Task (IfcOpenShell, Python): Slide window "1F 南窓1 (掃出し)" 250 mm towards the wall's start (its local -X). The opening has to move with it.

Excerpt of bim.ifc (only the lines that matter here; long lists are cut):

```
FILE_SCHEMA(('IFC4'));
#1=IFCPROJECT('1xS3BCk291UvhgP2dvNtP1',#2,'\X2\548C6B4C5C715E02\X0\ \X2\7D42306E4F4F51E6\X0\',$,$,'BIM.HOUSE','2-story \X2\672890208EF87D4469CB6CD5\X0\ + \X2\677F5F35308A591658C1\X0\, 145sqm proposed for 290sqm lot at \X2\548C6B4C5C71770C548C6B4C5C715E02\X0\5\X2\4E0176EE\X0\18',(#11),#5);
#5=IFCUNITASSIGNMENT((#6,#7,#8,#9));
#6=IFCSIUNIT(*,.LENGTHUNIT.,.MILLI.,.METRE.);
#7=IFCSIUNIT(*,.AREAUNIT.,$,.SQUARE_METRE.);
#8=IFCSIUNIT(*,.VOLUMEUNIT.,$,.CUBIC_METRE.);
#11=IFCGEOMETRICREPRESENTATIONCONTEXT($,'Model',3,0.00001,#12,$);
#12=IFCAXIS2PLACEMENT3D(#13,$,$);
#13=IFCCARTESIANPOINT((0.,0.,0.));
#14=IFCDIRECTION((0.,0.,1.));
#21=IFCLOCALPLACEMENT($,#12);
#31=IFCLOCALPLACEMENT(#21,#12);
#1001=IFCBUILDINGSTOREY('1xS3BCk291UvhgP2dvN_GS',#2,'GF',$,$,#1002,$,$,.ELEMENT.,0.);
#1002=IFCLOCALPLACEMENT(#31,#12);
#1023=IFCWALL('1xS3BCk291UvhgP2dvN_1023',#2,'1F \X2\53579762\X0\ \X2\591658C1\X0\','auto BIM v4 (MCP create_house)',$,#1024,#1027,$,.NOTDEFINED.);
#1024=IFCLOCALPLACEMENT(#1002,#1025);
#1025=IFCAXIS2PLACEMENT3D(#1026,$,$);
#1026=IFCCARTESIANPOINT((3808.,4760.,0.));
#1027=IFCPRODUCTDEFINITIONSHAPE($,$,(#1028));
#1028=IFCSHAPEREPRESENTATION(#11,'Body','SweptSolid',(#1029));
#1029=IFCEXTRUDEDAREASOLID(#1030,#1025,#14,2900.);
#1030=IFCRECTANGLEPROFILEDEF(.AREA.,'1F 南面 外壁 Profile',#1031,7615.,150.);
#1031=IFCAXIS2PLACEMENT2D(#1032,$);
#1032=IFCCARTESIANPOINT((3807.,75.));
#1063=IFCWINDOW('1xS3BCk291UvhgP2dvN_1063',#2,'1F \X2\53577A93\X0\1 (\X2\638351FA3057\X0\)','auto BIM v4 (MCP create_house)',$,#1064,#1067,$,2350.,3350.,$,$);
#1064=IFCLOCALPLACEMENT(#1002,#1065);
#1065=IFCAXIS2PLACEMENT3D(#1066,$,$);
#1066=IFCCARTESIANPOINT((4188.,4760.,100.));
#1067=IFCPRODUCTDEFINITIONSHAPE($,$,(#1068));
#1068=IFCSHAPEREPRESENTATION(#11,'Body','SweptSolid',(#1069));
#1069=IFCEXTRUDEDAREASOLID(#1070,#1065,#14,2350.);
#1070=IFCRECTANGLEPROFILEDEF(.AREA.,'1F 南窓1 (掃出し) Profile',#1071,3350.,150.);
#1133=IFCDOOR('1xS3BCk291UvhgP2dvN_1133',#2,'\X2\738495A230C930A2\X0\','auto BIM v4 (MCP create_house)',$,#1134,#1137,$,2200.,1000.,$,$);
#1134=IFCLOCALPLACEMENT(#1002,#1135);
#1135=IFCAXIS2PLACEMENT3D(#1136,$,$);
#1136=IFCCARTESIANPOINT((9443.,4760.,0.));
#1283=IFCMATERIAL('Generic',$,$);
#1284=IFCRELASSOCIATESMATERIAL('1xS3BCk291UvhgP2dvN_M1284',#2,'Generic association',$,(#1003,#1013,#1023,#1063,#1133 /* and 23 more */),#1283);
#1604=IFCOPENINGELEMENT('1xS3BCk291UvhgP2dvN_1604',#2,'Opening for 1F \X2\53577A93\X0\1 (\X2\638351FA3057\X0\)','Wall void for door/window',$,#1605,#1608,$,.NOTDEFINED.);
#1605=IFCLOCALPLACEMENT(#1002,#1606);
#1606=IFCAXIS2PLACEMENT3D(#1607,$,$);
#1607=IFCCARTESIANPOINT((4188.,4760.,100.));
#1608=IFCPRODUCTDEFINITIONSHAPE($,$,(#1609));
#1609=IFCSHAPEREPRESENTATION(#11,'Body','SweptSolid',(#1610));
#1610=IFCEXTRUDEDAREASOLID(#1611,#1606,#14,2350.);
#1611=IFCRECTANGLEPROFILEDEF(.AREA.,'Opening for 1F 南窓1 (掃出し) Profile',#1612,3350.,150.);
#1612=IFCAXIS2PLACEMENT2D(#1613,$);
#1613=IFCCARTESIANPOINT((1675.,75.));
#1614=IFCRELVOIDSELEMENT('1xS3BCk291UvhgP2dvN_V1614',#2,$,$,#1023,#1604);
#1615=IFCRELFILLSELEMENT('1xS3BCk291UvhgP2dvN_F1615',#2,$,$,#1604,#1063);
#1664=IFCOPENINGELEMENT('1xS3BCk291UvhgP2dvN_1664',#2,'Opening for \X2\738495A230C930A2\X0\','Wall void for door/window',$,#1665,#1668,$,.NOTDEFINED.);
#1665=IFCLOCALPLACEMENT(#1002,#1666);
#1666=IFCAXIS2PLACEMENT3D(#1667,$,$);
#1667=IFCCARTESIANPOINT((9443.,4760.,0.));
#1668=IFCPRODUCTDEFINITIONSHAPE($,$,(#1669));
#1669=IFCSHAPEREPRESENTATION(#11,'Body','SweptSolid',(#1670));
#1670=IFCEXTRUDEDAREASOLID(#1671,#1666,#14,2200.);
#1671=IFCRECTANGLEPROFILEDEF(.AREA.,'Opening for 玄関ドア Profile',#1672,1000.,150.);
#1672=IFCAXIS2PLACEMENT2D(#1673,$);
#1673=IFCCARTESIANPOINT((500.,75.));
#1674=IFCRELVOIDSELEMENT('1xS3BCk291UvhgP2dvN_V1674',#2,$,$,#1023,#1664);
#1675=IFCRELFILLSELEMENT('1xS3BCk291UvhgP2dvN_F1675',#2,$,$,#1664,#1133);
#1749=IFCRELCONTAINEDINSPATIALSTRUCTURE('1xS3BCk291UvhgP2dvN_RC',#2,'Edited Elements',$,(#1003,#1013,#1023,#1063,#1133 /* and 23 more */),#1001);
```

```python
import ifcopenshell
import ifcopenshell.api.geometry
import ifcopenshell.util.placement
import ifcopenshell.util.unit

model = ifcopenshell.open("bim.ifc")
unit_scale = ifcopenshell.util.unit.calculate_unit_scale(model)

window = model.by_guid("1xS3BCk291UvhgP2dvN_1063")
opening = window.FillsVoids[0].RelatingOpeningElement
wall = opening.VoidsElements[0].RelatingBuildingElement

wall_matrix = ifcopenshell.util.placement.get_local_placement(wall.ObjectPlacement)
shift = wall_matrix[:3, 0] * -0.25 / unit_scale
before = ifcopenshell.util.placement.get_local_placement(window.ObjectPlacement)[:3, 3].copy()

# The window is not placed relative to its opening, so move both.
for product in (opening, window):
    matrix = ifcopenshell.util.placement.get_local_placement(product.ObjectPlacement)
    matrix[:3, 3] += shift
    ifcopenshell.api.geometry.edit_object_placement(model, product=product, matrix=matrix, is_si=False)

after = ifcopenshell.util.placement.get_local_placement(window.ObjectPlacement)[:3, 3]
print("window moved by", (after - before).round(3) + 0.0)

model.write("bim_updated.ifc")
```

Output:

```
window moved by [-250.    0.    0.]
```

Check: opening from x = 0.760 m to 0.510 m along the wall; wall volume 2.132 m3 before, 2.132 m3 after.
